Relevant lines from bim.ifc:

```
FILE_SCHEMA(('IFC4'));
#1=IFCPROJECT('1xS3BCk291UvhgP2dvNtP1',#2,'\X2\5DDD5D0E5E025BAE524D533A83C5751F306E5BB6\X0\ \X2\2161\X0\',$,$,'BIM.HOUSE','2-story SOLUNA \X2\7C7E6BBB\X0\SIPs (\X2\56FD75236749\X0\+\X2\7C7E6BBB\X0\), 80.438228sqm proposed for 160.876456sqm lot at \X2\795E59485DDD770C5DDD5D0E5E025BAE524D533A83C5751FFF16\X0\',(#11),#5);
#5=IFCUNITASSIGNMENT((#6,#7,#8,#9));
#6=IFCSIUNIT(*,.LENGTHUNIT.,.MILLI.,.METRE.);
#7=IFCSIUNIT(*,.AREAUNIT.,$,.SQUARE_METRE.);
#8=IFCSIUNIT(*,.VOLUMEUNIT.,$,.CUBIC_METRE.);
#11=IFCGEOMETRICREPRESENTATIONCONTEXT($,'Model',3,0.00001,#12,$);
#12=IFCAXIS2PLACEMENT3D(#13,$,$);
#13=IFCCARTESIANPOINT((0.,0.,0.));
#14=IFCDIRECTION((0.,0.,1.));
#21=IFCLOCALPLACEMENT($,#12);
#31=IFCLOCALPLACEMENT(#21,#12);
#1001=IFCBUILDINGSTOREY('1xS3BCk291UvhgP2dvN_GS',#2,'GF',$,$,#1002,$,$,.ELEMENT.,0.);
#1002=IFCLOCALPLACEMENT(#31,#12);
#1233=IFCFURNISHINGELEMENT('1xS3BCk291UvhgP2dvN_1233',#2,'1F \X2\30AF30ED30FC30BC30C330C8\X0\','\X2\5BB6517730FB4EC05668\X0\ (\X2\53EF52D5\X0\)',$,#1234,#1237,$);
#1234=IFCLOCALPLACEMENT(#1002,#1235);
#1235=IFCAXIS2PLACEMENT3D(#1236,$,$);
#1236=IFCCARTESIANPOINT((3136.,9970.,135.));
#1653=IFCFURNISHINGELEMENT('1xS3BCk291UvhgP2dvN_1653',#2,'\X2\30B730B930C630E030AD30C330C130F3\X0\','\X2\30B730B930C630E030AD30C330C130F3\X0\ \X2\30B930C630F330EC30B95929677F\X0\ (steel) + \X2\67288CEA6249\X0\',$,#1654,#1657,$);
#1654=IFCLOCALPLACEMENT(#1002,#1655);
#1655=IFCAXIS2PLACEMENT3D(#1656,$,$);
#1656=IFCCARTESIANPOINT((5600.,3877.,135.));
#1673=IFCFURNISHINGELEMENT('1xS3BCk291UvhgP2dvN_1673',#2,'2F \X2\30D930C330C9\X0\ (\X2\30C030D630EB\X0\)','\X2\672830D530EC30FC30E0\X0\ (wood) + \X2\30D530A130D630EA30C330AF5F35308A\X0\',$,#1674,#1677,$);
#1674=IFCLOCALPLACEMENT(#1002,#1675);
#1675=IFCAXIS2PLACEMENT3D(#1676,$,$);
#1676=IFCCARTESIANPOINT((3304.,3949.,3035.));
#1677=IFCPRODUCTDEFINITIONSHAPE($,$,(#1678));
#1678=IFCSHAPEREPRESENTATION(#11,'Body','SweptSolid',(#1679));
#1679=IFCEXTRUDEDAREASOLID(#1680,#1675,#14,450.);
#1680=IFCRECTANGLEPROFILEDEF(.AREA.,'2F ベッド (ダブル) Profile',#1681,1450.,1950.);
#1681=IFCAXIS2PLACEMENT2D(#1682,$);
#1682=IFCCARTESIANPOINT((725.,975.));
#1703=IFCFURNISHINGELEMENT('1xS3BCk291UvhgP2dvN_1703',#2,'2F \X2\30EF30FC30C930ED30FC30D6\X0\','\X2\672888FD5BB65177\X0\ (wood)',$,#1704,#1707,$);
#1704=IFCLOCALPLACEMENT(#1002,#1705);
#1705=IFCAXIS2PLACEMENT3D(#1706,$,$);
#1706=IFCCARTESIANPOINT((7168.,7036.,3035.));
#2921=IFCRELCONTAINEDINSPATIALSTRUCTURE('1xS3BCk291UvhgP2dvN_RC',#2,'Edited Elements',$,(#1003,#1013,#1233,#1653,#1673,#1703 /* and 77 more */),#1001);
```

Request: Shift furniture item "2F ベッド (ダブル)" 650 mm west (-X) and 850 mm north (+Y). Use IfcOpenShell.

```python
import ifcopenshell
import ifcopenshell.api.geometry
import ifcopenshell.util.placement
import ifcopenshell.util.unit

model = ifcopenshell.open("bim.ifc")
unit_scale = ifcopenshell.util.unit.calculate_unit_scale(model)

item = model.by_guid("1xS3BCk291UvhgP2dvN_1673")
matrix = ifcopenshell.util.placement.get_local_placement(item.ObjectPlacement)
matrix[0, 3] -= 0.65 / unit_scale
matrix[1, 3] += 0.85 / unit_scale
ifcopenshell.api.geometry.edit_object_placement(model, product=item, matrix=matrix, is_si=False)

print(ifcopenshell.util.placement.get_local_placement(item.ObjectPlacement).round(3) + 0.0)

model.write("bim_edited.ifc")
```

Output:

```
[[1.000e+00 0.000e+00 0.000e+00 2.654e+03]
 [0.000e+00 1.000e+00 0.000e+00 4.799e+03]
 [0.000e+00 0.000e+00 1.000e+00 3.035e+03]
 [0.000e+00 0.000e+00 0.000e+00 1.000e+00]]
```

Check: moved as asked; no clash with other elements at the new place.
